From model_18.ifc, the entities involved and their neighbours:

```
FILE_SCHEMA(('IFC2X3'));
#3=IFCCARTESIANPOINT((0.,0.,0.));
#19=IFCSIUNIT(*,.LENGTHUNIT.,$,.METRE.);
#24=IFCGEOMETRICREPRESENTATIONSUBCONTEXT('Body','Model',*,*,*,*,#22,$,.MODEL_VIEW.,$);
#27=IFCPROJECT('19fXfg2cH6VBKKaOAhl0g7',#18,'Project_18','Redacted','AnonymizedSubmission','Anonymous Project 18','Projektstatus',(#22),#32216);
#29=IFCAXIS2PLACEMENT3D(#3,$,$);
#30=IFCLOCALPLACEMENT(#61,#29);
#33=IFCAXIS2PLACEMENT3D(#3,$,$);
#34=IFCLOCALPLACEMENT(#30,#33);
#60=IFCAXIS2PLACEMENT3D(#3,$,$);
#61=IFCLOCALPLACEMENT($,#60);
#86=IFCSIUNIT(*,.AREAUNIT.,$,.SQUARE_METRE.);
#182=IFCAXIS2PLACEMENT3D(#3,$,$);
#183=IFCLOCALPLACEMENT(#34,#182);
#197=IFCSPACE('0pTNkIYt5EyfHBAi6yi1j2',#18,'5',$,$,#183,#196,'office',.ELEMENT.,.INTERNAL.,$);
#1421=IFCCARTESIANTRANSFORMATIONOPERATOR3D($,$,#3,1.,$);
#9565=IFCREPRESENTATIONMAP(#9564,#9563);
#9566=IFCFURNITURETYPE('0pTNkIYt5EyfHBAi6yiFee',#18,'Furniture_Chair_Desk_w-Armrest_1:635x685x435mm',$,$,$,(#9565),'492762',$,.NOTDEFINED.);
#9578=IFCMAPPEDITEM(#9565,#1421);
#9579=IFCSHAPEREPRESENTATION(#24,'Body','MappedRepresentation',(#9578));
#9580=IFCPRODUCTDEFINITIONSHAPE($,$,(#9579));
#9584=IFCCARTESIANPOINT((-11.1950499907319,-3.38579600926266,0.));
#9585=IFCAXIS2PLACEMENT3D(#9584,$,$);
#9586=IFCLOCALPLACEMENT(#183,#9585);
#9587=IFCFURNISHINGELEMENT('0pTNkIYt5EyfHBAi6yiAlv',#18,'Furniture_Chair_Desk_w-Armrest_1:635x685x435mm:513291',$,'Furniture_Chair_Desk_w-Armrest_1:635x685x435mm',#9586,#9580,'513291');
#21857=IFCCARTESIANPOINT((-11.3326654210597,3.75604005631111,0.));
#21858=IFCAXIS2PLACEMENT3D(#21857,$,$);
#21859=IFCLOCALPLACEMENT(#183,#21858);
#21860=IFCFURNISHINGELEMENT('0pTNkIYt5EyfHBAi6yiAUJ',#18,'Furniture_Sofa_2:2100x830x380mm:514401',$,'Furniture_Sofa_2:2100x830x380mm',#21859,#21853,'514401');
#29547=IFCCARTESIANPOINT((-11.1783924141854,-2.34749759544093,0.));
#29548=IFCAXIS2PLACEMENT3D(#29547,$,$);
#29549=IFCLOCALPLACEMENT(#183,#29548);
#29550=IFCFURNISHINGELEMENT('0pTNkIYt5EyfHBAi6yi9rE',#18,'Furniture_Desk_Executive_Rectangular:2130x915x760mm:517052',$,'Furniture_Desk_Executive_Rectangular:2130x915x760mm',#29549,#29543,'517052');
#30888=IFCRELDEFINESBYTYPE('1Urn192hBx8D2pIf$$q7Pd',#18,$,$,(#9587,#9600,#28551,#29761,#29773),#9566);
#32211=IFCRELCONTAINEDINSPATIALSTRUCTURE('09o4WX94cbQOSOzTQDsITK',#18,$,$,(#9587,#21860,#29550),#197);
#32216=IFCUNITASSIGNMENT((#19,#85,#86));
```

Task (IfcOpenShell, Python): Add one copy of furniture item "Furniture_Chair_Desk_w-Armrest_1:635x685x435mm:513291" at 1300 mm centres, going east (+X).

```python
import numpy as np
import ifcopenshell
import ifcopenshell.api.geometry
import ifcopenshell.api.root
import ifcopenshell.util.element
import ifcopenshell.util.placement

model = ifcopenshell.open("model_18.ifc")


def reuse_history(source, copy):
    """copy_class also copies each property set's owner history, people and application; keep the originals."""
    for rel in copy.IsDefinedBy:
        if rel.is_a("IfcRelDefinesByProperties") and (history := rel.RelatingPropertyDefinition.OwnerHistory):
            rel.RelatingPropertyDefinition.OwnerHistory = source.OwnerHistory
            ifcopenshell.util.element.remove_deep2(model, history)


source = model.by_guid("0pTNkIYt5EyfHBAi6yiAlv")
base = ifcopenshell.util.placement.get_local_placement(source.ObjectPlacement)
step = np.array([1.0, 0.0, 0.0]) * 1.3

for i in range(1, 2):
    copy = ifcopenshell.api.root.copy_class(model, product=source)
    copy.Representation = ifcopenshell.util.element.copy_deep(
        model, source.Representation, exclude=["IfcGeometricRepresentationContext", "IfcRepresentationMap"]
    )
    copy.Name = "Furniture_Chair_Desk_w-Armrest_1:635x685x435mm"
    copy.Tag = None
    reuse_history(source, copy)
    matrix = base.copy()
    matrix[:3, 3] += i * step
    print("added at", matrix[:3, 3].round(3) + 0.0)
    ifcopenshell.api.geometry.edit_object_placement(model, product=copy, matrix=matrix, is_si=False)

model.write("model_18-out.ifc")
```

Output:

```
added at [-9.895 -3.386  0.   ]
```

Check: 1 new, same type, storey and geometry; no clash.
